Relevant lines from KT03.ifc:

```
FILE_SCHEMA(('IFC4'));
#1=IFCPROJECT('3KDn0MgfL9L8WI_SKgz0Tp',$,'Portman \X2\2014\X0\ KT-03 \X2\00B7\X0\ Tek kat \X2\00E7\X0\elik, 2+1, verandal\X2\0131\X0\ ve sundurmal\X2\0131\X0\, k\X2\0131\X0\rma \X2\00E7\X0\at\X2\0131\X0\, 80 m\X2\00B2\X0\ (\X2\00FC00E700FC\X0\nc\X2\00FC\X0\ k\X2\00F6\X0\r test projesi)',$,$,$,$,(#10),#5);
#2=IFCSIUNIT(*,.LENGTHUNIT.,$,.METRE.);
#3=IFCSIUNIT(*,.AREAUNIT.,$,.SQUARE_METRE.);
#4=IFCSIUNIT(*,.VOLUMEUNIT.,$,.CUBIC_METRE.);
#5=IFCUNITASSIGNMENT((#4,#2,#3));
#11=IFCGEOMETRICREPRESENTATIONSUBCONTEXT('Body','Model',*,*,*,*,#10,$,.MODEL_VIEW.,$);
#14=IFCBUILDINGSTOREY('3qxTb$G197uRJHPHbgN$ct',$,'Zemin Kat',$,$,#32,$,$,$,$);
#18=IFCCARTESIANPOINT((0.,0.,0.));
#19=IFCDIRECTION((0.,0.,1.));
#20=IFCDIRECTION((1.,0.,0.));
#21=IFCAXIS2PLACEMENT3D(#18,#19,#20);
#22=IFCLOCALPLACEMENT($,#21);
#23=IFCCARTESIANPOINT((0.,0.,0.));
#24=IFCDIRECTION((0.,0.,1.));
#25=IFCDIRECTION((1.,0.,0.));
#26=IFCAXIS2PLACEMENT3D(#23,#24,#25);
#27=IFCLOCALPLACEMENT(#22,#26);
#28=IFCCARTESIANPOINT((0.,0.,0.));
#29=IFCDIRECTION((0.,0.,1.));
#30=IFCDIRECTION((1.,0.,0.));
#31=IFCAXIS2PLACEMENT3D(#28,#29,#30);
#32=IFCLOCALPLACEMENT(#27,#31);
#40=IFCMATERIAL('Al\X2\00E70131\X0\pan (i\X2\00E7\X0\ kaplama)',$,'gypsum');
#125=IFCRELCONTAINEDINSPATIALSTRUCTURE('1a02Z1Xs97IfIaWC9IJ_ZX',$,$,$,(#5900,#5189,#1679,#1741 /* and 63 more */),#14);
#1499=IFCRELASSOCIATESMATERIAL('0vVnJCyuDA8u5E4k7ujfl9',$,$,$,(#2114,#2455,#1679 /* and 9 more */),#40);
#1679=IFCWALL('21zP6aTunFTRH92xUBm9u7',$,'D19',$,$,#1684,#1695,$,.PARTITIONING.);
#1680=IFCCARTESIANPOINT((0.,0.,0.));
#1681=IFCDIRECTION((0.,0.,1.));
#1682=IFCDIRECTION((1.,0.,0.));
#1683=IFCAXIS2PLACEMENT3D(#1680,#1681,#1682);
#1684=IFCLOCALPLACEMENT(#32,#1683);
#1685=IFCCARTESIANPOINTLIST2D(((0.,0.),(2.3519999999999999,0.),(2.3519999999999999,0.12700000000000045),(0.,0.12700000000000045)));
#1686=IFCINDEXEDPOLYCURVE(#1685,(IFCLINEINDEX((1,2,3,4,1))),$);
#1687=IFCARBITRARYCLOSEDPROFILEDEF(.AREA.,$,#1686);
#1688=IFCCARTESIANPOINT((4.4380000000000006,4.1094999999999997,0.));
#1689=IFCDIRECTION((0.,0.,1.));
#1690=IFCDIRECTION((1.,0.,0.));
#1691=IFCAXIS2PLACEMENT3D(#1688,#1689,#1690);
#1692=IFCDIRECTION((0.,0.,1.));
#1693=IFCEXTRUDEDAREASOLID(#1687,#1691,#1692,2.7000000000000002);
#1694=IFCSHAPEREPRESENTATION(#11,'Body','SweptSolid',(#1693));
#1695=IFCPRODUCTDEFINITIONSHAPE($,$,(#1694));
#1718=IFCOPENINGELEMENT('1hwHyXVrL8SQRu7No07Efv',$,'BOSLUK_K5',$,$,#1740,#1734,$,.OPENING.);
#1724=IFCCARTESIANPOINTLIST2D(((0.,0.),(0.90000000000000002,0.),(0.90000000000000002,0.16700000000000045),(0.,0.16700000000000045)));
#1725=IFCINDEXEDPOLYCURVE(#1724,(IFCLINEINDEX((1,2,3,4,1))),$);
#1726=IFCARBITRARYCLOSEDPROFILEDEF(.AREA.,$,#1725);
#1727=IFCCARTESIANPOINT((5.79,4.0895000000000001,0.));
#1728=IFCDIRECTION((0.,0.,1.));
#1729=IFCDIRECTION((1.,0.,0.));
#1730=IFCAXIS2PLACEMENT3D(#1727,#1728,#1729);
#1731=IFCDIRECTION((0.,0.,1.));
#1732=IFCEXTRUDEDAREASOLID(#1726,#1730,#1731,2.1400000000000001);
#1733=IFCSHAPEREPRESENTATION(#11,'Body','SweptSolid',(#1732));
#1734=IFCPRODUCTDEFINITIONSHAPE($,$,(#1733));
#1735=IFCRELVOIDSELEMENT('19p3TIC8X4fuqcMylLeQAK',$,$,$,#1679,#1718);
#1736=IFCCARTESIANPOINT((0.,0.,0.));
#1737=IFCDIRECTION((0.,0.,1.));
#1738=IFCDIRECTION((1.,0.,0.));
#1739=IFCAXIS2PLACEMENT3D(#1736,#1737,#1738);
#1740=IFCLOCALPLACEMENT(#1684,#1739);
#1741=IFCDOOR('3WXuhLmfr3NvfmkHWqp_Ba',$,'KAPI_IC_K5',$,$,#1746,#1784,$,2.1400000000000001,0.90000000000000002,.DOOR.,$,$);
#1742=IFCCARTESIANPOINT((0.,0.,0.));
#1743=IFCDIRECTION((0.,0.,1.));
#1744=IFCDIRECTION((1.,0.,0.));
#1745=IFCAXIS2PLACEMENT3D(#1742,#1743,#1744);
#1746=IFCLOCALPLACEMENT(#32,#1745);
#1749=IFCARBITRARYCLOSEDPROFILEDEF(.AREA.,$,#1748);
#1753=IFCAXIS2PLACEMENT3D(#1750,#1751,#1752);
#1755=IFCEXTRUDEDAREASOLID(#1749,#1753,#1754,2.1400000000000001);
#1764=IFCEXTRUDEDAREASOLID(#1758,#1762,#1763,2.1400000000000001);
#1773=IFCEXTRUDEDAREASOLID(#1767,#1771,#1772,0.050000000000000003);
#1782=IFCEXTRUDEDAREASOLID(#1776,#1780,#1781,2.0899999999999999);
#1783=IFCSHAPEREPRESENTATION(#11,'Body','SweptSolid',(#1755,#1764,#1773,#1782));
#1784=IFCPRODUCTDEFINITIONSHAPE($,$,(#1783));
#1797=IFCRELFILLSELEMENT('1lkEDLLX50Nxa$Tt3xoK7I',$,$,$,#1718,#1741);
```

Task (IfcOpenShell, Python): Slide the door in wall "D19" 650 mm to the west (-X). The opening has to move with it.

```python
import ifcopenshell
import ifcopenshell.api.geometry
import ifcopenshell.util.placement

model = ifcopenshell.open("KT03.ifc")

door = model.by_guid("3WXuhLmfr3NvfmkHWqp_Ba")
opening = door.FillsVoids[0].RelatingOpeningElement
wall = opening.VoidsElements[0].RelatingBuildingElement

wall_matrix = ifcopenshell.util.placement.get_local_placement(wall.ObjectPlacement)
shift = wall_matrix[:3, 0] * -0.65
before = ifcopenshell.util.placement.get_local_placement(door.ObjectPlacement)[:3, 3].copy()

# The door is not placed relative to its opening, so move both.
for product in (opening, door):
    matrix = ifcopenshell.util.placement.get_local_placement(product.ObjectPlacement)
    matrix[:3, 3] += shift
    ifcopenshell.api.geometry.edit_object_placement(model, product=product, matrix=matrix, is_si=False)

after = ifcopenshell.util.placement.get_local_placement(door.ObjectPlacement)[:3, 3]
print("door moved by", (after - before).round(3) + 0.0)

model.write("KT03_updated.ifc")
```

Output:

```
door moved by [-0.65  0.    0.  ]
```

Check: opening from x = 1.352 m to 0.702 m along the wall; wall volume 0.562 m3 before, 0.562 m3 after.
